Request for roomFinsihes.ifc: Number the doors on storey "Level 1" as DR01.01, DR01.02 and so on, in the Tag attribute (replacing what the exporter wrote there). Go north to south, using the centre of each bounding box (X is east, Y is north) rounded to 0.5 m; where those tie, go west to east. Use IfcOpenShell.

First a look at what the model holds.

```python
import ifcopenshell
import ifcopenshell.util.element
import ifcopenshell.util.placement

model = ifcopenshell.open("roomFinsihes.ifc")
print(model.schema)
storey = next(s for s in model.by_type("IfcBuildingStorey") if s.Name == "Level 1")
doors = [e for e in ifcopenshell.util.element.get_decomposition(storey) if e.is_a("IfcDoor")]
for e in sorted(doors, key=lambda e: e.id()):
    origin = ifcopenshell.util.placement.get_local_placement(e.ObjectPlacement)[:3, 3]
    print(e.id(), e.Tag, e.Name, origin.round(2) + 0.0, sep=" | ")
```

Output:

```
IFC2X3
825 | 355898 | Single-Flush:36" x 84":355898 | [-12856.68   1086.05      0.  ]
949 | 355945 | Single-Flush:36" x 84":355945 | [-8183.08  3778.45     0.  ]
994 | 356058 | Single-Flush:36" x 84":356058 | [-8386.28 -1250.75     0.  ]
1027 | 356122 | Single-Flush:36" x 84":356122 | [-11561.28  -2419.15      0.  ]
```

```python
import ifcopenshell
import ifcopenshell.geom
import ifcopenshell.util.element
import ifcopenshell.util.shape

model = ifcopenshell.open("roomFinsihes.ifc")
settings = ifcopenshell.geom.settings()
settings.set("use-world-coords", True)


def centre(element):
    shape = ifcopenshell.geom.create_shape(settings, element)
    return ifcopenshell.util.shape.get_bbox_centroid(shape.geometry)


storey = next(s for s in model.by_type("IfcBuildingStorey") if s.Name == "Level 1")
doors = [e for e in ifcopenshell.util.element.get_decomposition(storey) if e.is_a("IfcDoor")]

# Insertion points can sit at a corner or the storey origin, so sort by the geometry (in metres).
centres = {e: centre(e) for e in doors}
doors.sort(key=lambda e: (-round(centres[e][1] / 0.5), centres[e][0]))

for i, e in enumerate(doors, start=1):
    number = f"DR01.{i:02d}"
    e.Tag = number
    print(e.id(), number)

model.write("roomFinsihes_edited.ifc")
```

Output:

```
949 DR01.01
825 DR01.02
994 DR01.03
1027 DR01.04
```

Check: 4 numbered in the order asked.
